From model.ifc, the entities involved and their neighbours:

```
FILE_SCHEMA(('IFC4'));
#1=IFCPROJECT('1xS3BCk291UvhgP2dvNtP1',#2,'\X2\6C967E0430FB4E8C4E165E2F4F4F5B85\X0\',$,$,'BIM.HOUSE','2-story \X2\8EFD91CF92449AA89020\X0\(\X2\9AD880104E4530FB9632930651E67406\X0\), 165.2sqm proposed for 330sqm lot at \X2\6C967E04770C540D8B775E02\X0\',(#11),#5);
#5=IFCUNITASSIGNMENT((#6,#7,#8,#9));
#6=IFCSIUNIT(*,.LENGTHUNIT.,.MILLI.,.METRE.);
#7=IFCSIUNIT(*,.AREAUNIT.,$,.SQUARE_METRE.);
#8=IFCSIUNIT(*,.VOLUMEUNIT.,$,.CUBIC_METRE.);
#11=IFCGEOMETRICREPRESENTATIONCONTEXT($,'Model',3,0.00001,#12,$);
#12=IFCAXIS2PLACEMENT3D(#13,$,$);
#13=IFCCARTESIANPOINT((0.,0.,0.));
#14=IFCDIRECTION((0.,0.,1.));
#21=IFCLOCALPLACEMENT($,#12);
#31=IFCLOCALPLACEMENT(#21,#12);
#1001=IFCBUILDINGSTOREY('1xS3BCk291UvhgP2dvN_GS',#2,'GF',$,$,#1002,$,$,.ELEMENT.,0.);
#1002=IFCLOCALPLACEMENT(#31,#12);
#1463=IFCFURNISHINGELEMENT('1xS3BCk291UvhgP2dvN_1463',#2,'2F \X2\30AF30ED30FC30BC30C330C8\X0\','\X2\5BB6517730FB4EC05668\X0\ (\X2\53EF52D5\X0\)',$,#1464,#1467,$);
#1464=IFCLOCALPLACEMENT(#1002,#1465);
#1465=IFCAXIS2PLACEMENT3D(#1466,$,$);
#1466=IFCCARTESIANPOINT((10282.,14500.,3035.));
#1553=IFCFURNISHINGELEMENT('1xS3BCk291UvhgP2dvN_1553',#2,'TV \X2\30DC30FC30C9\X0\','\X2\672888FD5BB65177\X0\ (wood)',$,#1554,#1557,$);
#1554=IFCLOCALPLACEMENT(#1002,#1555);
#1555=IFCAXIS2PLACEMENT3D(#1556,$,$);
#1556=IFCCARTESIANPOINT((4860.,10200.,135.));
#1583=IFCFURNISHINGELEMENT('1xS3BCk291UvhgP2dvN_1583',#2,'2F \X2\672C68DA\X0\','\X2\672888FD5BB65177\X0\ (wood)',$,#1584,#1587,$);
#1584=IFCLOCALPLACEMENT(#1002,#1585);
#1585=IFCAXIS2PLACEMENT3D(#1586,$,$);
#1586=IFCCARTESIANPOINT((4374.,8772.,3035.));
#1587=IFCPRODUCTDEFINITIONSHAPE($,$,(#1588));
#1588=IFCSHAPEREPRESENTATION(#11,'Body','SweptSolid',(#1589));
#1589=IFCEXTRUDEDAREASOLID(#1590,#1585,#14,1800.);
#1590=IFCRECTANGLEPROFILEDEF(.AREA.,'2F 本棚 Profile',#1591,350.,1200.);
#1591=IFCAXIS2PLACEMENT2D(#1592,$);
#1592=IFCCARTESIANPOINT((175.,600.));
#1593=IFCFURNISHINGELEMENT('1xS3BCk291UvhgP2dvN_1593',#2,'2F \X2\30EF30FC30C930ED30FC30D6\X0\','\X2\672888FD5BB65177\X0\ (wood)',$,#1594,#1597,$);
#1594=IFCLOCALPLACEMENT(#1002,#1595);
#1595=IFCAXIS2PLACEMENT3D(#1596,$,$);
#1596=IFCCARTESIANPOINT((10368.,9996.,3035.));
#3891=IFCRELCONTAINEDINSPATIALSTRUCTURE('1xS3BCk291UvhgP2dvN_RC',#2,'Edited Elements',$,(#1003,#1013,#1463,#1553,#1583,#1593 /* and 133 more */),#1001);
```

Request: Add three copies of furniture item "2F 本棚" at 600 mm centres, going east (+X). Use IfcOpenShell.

```python
import numpy as np
import ifcopenshell
import ifcopenshell.api.geometry
import ifcopenshell.api.root
import ifcopenshell.util.element
import ifcopenshell.util.placement

model = ifcopenshell.open("model.ifc")


def reuse_history(source, copy):
    """copy_class also copies each property set's owner history, people and application; keep the originals."""
    for rel in copy.IsDefinedBy:
        if rel.is_a("IfcRelDefinesByProperties") and (history := rel.RelatingPropertyDefinition.OwnerHistory):
            rel.RelatingPropertyDefinition.OwnerHistory = source.OwnerHistory
            ifcopenshell.util.element.remove_deep2(model, history)


source = model.by_guid("1xS3BCk291UvhgP2dvN_1583")
base = ifcopenshell.util.placement.get_local_placement(source.ObjectPlacement)
step = np.array([1.0, 0.0, 0.0]) * 600.0

for i in range(1, 4):
    copy = ifcopenshell.api.root.copy_class(model, product=source)
    copy.Representation = ifcopenshell.util.element.copy_deep(
        model, source.Representation, exclude=["IfcGeometricRepresentationContext", "IfcRepresentationMap"]
    )
    reuse_history(source, copy)
    matrix = base.copy()
    matrix[:3, 3] += i * step
    print("added at", matrix[:3, 3].round(3) + 0.0)
    ifcopenshell.api.geometry.edit_object_placement(model, product=copy, matrix=matrix, is_si=False)

model.write("model_edited.ifc")
```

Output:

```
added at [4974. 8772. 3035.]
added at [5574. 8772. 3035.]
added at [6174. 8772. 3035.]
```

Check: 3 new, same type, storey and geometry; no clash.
